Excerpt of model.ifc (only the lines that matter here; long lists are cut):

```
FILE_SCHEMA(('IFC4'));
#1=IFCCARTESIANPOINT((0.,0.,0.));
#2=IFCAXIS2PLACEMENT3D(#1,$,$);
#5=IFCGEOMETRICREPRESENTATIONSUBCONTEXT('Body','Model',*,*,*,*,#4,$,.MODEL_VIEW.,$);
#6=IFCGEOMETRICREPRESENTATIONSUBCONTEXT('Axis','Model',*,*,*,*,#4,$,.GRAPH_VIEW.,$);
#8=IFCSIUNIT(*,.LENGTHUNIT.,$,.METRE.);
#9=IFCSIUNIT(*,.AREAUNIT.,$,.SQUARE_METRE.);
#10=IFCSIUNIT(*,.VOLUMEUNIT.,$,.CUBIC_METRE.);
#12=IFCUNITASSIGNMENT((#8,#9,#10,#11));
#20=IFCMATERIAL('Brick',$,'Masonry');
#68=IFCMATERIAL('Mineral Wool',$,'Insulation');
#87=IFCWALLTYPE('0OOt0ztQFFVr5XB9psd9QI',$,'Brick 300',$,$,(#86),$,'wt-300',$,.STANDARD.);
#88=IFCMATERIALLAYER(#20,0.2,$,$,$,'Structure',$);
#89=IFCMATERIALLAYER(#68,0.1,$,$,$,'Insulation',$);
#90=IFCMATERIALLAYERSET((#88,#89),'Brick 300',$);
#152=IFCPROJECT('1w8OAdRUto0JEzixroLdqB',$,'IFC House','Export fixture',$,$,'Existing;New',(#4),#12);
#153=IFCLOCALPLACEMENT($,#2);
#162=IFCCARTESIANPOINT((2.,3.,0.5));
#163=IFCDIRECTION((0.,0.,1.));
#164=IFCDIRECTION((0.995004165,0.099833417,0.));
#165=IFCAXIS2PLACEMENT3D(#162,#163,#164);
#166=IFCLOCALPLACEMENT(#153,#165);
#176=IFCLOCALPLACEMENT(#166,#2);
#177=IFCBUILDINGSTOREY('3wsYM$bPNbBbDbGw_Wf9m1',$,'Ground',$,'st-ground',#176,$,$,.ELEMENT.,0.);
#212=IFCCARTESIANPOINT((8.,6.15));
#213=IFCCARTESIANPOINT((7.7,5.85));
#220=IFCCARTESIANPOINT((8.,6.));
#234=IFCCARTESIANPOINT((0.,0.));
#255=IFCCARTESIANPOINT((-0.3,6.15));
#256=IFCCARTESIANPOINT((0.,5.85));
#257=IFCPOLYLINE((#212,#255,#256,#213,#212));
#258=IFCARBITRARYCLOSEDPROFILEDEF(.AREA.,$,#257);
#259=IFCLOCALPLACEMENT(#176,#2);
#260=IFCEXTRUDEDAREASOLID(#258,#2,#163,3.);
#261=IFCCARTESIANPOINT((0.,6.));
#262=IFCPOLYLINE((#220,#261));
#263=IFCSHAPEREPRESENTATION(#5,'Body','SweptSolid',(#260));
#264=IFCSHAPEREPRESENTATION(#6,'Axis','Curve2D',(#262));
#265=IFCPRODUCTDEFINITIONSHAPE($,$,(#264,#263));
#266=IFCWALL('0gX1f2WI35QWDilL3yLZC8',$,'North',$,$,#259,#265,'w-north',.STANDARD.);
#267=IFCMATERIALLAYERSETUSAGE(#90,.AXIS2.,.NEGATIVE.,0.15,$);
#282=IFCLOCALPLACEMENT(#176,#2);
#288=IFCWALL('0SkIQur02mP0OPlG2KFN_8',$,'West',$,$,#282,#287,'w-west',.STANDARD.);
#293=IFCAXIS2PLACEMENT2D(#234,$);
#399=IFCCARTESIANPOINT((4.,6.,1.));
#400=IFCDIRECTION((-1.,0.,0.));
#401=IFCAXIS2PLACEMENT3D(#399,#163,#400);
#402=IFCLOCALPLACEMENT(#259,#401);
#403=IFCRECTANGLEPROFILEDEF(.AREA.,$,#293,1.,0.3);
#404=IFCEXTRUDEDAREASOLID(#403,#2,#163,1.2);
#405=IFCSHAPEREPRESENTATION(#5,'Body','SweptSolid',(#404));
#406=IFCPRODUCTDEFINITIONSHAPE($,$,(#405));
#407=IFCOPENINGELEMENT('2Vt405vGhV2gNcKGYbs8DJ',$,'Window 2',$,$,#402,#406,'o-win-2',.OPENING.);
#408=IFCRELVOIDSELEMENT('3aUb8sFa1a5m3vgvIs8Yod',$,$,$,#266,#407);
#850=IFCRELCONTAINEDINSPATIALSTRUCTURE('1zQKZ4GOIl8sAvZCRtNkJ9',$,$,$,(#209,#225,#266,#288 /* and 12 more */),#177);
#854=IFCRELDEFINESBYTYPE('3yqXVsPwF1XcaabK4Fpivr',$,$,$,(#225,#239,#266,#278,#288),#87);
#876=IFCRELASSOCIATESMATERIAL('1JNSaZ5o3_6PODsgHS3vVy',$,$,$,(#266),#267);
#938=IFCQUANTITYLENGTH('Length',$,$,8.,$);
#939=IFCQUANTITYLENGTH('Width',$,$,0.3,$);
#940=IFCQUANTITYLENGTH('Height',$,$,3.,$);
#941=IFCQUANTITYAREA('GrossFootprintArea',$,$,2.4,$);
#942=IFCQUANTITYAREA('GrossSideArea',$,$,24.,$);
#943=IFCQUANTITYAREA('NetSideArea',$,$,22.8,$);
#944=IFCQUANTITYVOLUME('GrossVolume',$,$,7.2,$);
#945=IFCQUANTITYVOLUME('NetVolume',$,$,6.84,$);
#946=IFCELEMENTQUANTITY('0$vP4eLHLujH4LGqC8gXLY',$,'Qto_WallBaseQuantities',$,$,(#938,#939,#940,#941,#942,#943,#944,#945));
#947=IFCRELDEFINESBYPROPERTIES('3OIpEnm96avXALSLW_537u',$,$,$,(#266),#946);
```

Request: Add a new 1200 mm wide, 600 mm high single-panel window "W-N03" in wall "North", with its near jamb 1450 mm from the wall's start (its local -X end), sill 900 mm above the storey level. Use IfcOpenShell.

```python
import numpy as np
import ifcopenshell
import ifcopenshell.api.feature
import ifcopenshell.api.geometry
import ifcopenshell.api.pset
import ifcopenshell.api.root
import ifcopenshell.api.spatial
import ifcopenshell.geom
import ifcopenshell.util.element
import ifcopenshell.util.placement
import ifcopenshell.util.representation
import ifcopenshell.util.shape
import ifcopenshell.util.unit

model = ifcopenshell.open("model.ifc")
unit_scale = ifcopenshell.util.unit.calculate_unit_scale(model)
area_scale = ifcopenshell.util.unit.calculate_unit_scale(model, "AREAUNIT")
volume_scale = ifcopenshell.util.unit.calculate_unit_scale(model, "VOLUMEUNIT")
settings = ifcopenshell.geom.settings()


def volume(element):
    """Net volume in cubic metres, openings subtracted."""
    shape = ifcopenshell.geom.create_shape(settings, element)
    return ifcopenshell.util.shape.get_volume(shape.geometry)


wall = model.by_id(266)
storey = ifcopenshell.util.element.get_container(wall, ifc_class="IfcBuildingStorey")
context = ifcopenshell.util.representation.get_context(model, "Model", "Body", "MODEL_VIEW")
before = volume(wall)

width, height, from_end, sill = 1.2, 0.6, 1.45, 0.9  # metres

# The wall runs along its own X axis, and the end named is its -X end.
wall_shape = ifcopenshell.geom.create_shape(settings, wall)
x, y, z = ifcopenshell.util.shape.get_vertices(wall_shape.geometry).T
start = x.min() + from_end
face, thickness = float(y.min()), float(y.max() - y.min())
wall_matrix = ifcopenshell.util.placement.get_local_placement(wall.ObjectPlacement)
level = ifcopenshell.util.placement.get_local_placement(storey.ObjectPlacement)[2, 3]


def in_wall(x, y):
    """Placement at x, y metres in the wall's axes, at sill height."""
    matrix = wall_matrix.copy()
    matrix[:, 3] = wall_matrix @ np.array([x / unit_scale, y / unit_scale, 0.0, 1.0])
    matrix[2, 3] = level + sill / unit_scale
    return matrix


# Opening: a box that overshoots both wall faces by 50 mm.
opening = ifcopenshell.api.root.create_entity(model, ifc_class="IfcOpeningElement", predefined_type="OPENING")
box = ifcopenshell.api.geometry.add_wall_representation(
    model, context=context, length=width, height=height, thickness=thickness + 0.1
)
ifcopenshell.api.geometry.assign_representation(model, product=opening, representation=box)
ifcopenshell.api.geometry.edit_object_placement(model, product=opening, matrix=in_wall(start, face - 0.05), is_si=False)
ifcopenshell.api.feature.add_feature(model, feature=opening, element=wall)

window = ifcopenshell.api.root.create_entity(model, ifc_class="IfcWindow", name="W-N03", predefined_type="WINDOW")
window.OverallWidth, window.OverallHeight = width / unit_scale, height / unit_scale
window.PartitioningType = "SINGLE_PANEL"
body = ifcopenshell.api.geometry.add_window_representation(
    model,
    context=context,
    overall_width=window.OverallWidth,
    overall_height=window.OverallHeight,
    partition_type="SINGLE_PANEL",
)
ifcopenshell.api.geometry.assign_representation(model, product=window, representation=body)
ifcopenshell.api.spatial.assign_container(model, products=[window], relating_structure=storey)
ifcopenshell.api.feature.add_filling(model, opening=opening, element=window)

# Centre the window in the wall's thickness.
ifcopenshell.api.geometry.edit_object_placement(model, product=window, matrix=in_wall(start, face), is_si=False)
window_shape = ifcopenshell.geom.create_shape(settings, window)
depth = ifcopenshell.util.shape.get_vertices(window_shape.geometry)[:, 1]
offset = face + thickness / 2 - (depth.min() + depth.max()) / 2
ifcopenshell.api.geometry.edit_object_placement(model, product=window, matrix=in_wall(start, offset), is_si=False)

after = volume(wall)

# Update the wall's stored quantities.
qto = model.by_id(ifcopenshell.util.element.get_pset(wall, "Qto_WallBaseQuantities", should_inherit=False)["id"])
ifcopenshell.api.pset.edit_qto(model, qto=qto, properties={
    "NetSideArea": after / thickness / area_scale,
    "NetVolume": after / volume_scale,
})

print(f"wall volume {before:.3f} -> {after:.3f} m3")

model.write("model_v2.ifc")
```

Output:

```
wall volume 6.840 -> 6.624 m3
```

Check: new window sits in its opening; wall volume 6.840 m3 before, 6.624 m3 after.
